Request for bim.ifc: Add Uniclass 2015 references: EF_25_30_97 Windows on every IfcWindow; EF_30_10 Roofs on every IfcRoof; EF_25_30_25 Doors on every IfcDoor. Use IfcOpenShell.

First a look at what the model holds.

```python
import ifcopenshell

model = ifcopenshell.open("bim.ifc")
print(model.schema)
print("classifications:", [c.Name for c in model.by_type("IfcClassification")])
for ifc_class in ("IfcDoor", "IfcRoof", "IfcStair", "IfcWall", "IfcWindow"):
    print(ifc_class, len(model.by_type(ifc_class)))
```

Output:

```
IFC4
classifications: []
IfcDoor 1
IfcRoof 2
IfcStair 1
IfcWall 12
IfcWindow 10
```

```python
import ifcopenshell
import ifcopenshell.api.classification

model = ifcopenshell.open("bim.ifc")

system = ifcopenshell.api.classification.add_classification(model, classification="Uniclass 2015")

codes = {
    "IfcWindow": ("EF_25_30_97", "Windows"),
    "IfcRoof": ("EF_30_10", "Roofs"),
    "IfcDoor": ("EF_25_30_25", "Doors"),
}
for ifc_class, (code, name) in codes.items():
    products = model.by_type(ifc_class)
    ifcopenshell.api.classification.add_reference(
        model, products=products, classification=system, identification=code, name=name
    )
    print(code, len(products))

model.write("bim_v2.ifc")
```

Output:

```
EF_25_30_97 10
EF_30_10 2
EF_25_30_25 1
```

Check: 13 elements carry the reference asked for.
